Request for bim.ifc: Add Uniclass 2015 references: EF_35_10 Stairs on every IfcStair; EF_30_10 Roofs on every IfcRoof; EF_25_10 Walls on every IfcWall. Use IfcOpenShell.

First a look at what the model holds.

```python
import ifcopenshell

model = ifcopenshell.open("bim.ifc")
print(model.schema)
print("classifications:", [c.Name for c in model.by_type("IfcClassification")])
for ifc_class in ("IfcDoor", "IfcRoof", "IfcStair", "IfcWall", "IfcWindow"):
    print(ifc_class, len(model.by_type(ifc_class)))
```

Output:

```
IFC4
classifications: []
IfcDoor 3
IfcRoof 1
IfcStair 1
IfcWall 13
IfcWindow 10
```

```python
import ifcopenshell
import ifcopenshell.api.classification

model = ifcopenshell.open("bim.ifc")

system = ifcopenshell.api.classification.add_classification(model, classification="Uniclass 2015")

codes = {
    "IfcStair": ("EF_35_10", "Stairs"),
    "IfcRoof": ("EF_30_10", "Roofs"),
    "IfcWall": ("EF_25_10", "Walls"),
}
for ifc_class, (code, name) in codes.items():
    products = model.by_type(ifc_class)
    ifcopenshell.api.classification.add_reference(
        model, products=products, classification=system, identification=code, name=name
    )
    print(code, len(products))

model.write("bim_rev.ifc")
```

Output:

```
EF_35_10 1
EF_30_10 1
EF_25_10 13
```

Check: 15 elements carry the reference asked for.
